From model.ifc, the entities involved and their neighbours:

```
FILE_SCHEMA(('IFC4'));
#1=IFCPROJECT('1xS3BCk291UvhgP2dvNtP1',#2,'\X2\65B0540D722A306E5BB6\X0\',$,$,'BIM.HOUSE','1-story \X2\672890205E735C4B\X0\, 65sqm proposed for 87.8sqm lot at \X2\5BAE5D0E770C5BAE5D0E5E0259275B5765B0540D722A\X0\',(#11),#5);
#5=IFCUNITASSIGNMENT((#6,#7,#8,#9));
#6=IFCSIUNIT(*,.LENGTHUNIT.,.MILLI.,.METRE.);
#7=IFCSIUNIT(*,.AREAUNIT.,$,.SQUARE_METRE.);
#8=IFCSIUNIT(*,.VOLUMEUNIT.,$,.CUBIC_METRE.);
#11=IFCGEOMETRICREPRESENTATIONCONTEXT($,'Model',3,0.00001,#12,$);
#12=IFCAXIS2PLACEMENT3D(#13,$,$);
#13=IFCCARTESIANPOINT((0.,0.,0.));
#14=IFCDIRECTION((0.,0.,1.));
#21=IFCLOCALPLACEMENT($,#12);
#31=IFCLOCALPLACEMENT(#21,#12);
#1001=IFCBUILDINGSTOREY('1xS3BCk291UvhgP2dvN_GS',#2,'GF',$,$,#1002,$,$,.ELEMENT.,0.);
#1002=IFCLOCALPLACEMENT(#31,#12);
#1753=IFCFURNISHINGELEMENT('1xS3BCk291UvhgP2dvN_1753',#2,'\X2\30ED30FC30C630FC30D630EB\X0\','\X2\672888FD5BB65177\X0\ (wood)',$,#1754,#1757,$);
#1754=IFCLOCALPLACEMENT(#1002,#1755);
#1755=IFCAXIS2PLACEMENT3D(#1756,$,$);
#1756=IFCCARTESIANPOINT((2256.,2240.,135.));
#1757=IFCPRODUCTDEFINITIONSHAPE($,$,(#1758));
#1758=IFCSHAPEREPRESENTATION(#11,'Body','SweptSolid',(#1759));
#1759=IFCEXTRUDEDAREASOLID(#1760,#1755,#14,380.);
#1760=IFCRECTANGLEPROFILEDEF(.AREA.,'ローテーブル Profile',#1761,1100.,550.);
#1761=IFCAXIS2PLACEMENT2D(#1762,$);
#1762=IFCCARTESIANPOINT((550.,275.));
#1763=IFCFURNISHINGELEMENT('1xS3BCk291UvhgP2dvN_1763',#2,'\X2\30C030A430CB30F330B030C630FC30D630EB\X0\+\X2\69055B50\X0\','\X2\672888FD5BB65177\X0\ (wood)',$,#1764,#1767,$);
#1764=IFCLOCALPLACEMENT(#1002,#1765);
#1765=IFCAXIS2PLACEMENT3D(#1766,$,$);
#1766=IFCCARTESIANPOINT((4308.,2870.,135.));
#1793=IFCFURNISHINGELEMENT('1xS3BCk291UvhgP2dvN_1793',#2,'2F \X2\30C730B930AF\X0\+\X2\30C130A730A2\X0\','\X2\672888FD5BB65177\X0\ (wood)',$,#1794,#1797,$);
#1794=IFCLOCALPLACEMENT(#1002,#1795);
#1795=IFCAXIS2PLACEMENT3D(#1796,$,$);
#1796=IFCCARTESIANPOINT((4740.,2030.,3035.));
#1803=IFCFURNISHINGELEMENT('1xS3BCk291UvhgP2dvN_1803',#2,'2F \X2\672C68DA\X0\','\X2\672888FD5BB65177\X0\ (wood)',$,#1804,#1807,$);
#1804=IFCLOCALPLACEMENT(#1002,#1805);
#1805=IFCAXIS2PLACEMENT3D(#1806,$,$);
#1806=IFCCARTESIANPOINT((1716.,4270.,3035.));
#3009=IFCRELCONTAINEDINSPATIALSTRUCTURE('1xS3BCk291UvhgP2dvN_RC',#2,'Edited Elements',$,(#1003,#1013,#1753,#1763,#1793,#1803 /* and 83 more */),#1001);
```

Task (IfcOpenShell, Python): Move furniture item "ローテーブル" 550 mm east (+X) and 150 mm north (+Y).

```python
import ifcopenshell
import ifcopenshell.api.geometry
import ifcopenshell.util.placement
import ifcopenshell.util.unit

model = ifcopenshell.open("model.ifc")
unit_scale = ifcopenshell.util.unit.calculate_unit_scale(model)

item = model.by_guid("1xS3BCk291UvhgP2dvN_1753")
matrix = ifcopenshell.util.placement.get_local_placement(item.ObjectPlacement)
matrix[0, 3] += 0.55 / unit_scale
matrix[1, 3] += 0.15 / unit_scale
ifcopenshell.api.geometry.edit_object_placement(model, product=item, matrix=matrix, is_si=False)

print(ifcopenshell.util.placement.get_local_placement(item.ObjectPlacement).round(3) + 0.0)

model.write("model_edited.ifc")
```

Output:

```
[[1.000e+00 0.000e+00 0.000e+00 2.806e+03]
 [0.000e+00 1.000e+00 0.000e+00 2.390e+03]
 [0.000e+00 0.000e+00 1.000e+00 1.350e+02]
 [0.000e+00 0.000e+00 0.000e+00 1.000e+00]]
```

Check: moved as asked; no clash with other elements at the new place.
